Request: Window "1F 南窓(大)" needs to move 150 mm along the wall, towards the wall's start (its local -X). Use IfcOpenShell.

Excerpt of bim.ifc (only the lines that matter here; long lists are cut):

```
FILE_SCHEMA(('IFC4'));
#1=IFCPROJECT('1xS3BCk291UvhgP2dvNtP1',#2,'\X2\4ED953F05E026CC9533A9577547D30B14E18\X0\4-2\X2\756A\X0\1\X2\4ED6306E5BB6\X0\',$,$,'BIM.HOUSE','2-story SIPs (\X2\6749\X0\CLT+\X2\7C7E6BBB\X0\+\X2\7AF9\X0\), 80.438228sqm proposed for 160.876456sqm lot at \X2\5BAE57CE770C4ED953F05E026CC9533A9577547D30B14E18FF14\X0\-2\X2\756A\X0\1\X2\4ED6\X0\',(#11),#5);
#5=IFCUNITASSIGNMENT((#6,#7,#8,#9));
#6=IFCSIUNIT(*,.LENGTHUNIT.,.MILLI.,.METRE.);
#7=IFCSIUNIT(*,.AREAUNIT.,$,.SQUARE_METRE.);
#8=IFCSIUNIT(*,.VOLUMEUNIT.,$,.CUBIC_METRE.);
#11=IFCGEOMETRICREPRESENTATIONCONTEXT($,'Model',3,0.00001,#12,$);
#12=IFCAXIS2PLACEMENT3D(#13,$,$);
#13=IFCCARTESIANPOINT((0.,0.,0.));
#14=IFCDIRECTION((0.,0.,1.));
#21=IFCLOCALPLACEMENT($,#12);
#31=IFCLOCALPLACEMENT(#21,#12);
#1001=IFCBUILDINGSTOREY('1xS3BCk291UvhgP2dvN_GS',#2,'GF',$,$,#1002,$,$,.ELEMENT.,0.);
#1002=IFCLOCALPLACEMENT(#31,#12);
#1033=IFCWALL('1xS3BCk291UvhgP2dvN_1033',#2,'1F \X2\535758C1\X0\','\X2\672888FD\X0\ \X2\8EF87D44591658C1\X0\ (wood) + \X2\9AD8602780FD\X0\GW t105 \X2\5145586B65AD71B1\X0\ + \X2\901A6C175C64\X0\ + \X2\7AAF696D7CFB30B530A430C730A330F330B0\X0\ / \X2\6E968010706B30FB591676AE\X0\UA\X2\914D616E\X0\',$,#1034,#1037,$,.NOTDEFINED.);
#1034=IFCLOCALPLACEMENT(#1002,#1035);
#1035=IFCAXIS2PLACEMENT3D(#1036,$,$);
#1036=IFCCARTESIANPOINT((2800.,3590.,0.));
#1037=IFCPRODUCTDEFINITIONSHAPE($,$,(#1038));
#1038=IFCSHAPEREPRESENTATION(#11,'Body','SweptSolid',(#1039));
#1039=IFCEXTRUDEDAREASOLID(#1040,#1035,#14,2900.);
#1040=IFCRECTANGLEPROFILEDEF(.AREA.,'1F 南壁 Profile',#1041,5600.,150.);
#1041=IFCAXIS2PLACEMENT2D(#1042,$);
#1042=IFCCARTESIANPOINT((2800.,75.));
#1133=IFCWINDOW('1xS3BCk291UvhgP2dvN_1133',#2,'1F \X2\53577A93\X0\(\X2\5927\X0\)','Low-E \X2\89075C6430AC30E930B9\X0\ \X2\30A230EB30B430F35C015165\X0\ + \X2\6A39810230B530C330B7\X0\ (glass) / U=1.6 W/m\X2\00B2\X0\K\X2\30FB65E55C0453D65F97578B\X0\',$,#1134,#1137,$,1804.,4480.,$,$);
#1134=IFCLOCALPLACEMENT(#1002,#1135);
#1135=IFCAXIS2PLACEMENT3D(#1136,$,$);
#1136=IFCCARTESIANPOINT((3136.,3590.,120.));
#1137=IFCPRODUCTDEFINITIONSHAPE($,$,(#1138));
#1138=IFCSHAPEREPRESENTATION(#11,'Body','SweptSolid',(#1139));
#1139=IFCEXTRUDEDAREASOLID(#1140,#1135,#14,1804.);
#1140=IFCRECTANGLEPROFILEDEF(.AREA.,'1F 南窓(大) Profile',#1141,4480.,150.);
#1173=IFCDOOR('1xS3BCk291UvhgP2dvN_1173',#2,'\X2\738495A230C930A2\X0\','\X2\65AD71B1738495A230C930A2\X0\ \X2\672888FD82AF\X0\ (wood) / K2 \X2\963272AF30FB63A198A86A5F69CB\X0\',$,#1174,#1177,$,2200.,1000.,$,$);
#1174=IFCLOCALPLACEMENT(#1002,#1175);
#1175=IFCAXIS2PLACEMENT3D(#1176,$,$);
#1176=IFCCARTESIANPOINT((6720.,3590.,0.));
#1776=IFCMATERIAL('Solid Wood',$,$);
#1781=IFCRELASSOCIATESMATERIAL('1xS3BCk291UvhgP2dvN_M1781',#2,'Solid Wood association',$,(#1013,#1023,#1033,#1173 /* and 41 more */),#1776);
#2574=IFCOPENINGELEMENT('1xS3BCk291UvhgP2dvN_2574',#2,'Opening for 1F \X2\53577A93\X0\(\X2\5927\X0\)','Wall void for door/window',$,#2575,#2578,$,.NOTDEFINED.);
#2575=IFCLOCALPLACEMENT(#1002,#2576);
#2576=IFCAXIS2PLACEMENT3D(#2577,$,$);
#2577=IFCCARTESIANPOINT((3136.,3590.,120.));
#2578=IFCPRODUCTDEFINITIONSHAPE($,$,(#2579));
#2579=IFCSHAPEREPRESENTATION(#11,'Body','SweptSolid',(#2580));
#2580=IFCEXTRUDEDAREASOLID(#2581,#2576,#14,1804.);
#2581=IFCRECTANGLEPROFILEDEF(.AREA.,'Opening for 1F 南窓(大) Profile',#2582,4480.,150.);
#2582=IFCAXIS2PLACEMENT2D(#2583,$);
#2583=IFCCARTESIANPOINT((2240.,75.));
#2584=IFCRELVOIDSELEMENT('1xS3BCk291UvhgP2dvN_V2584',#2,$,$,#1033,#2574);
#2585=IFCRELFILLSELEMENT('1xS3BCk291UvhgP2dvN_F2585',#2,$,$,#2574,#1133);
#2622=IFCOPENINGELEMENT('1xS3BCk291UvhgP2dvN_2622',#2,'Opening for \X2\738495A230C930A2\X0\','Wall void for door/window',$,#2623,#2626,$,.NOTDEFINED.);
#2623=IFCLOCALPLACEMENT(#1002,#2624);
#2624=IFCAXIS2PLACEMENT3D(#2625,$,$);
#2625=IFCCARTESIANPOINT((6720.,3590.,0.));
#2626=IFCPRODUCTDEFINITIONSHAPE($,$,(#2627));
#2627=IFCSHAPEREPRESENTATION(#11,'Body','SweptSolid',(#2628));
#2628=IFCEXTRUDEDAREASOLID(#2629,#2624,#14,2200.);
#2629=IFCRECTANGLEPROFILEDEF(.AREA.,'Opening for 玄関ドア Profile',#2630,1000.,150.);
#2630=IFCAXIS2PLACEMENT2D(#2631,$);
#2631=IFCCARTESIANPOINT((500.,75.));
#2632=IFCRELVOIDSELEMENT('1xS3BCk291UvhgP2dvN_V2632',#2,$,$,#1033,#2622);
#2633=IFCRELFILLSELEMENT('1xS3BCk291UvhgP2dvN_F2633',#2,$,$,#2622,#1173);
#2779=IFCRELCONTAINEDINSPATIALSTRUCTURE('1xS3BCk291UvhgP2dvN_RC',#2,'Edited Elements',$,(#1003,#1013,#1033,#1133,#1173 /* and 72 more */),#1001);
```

```python
import ifcopenshell
import ifcopenshell.api.geometry
import ifcopenshell.util.placement

model = ifcopenshell.open("bim.ifc")

window = model.by_id(1133)
opening = window.FillsVoids[0].RelatingOpeningElement
wall = opening.VoidsElements[0].RelatingBuildingElement

wall_matrix = ifcopenshell.util.placement.get_local_placement(wall.ObjectPlacement)
shift = wall_matrix[:3, 0] * -150.0
before = ifcopenshell.util.placement.get_local_placement(window.ObjectPlacement)[:3, 3].copy()

# The window is not placed relative to its opening, so move both.
for product in (opening, window):
    matrix = ifcopenshell.util.placement.get_local_placement(product.ObjectPlacement)
    matrix[:3, 3] += shift
    ifcopenshell.api.geometry.edit_object_placement(model, product=product, matrix=matrix, is_si=False)

after = ifcopenshell.util.placement.get_local_placement(window.ObjectPlacement)[:3, 3]
print("window moved by", (after - before).round(3) + 0.0)

model.write("bim_rev.ifc")
```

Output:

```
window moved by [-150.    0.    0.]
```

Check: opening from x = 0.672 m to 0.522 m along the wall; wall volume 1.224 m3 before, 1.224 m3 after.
